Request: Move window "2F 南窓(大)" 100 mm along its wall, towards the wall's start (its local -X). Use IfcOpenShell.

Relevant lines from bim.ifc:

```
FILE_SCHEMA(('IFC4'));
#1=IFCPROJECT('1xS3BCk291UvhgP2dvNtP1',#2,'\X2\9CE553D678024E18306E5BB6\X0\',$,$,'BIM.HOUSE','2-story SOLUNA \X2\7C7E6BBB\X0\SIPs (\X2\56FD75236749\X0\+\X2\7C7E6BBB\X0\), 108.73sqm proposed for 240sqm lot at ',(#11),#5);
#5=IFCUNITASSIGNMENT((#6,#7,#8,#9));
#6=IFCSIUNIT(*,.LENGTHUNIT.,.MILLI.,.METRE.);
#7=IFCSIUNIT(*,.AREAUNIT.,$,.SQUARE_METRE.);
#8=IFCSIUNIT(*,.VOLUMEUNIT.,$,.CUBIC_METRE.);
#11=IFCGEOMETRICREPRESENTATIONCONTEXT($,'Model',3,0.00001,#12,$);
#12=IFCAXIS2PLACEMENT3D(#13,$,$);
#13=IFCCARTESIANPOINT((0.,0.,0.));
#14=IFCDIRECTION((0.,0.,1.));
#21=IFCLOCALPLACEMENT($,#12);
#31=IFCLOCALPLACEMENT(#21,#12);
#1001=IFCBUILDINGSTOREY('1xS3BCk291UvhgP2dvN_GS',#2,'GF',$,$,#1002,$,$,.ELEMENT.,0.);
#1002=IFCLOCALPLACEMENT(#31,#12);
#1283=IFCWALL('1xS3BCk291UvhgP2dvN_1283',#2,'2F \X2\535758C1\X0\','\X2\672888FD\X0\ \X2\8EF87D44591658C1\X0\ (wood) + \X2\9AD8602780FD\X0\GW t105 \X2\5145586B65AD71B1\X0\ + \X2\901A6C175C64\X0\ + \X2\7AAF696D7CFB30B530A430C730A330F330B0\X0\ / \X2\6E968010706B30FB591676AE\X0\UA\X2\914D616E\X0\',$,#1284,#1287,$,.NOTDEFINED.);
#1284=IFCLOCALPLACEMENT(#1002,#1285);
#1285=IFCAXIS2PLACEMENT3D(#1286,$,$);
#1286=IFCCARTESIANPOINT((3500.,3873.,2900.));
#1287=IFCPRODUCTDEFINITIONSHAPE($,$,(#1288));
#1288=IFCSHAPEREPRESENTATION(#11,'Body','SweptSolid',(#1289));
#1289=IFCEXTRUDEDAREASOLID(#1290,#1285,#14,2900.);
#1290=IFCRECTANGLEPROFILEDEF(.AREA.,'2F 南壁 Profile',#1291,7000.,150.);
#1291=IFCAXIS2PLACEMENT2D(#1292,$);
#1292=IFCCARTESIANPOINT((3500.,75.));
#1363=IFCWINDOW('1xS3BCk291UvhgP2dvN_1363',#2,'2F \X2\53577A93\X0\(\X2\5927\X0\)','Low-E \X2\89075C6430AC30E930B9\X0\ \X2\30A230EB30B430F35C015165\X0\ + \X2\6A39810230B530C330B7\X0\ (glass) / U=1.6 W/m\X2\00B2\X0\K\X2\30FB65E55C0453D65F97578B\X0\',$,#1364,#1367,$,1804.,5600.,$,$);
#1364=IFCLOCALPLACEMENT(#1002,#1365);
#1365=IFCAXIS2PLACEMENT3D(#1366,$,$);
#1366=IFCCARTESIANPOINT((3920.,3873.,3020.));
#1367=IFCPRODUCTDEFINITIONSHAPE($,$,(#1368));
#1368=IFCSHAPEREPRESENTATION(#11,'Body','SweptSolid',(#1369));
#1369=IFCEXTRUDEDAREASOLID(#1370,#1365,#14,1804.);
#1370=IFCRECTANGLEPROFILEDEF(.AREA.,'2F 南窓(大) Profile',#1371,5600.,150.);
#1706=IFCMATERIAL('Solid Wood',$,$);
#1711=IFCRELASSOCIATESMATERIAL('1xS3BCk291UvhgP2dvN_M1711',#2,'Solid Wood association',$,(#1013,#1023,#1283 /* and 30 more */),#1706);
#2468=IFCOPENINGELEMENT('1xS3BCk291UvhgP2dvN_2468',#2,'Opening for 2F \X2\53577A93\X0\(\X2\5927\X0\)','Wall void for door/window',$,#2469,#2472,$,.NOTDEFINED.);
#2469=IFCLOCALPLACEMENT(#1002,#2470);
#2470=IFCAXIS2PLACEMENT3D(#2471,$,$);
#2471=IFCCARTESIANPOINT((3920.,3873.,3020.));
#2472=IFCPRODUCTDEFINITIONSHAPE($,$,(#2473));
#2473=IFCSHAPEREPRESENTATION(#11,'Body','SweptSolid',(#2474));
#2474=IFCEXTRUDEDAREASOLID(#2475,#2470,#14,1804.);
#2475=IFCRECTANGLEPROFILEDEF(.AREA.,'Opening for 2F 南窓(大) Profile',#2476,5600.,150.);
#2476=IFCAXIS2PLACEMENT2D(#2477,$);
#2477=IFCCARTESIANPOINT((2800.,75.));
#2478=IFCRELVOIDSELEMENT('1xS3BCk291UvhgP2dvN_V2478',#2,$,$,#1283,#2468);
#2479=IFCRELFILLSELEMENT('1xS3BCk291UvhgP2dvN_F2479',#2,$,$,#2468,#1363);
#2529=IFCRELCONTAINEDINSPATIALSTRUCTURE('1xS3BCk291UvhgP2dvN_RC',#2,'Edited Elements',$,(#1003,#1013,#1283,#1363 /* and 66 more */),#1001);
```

```python
import ifcopenshell
import ifcopenshell.api.geometry
import ifcopenshell.util.placement

model = ifcopenshell.open("bim.ifc")

window = model.by_guid("1xS3BCk291UvhgP2dvN_1363")
opening = window.FillsVoids[0].RelatingOpeningElement
wall = opening.VoidsElements[0].RelatingBuildingElement

wall_matrix = ifcopenshell.util.placement.get_local_placement(wall.ObjectPlacement)
shift = wall_matrix[:3, 0] * -100.0
before = ifcopenshell.util.placement.get_local_placement(window.ObjectPlacement)[:3, 3].copy()

# The window is not placed relative to its opening, so move both.
for product in (opening, window):
    matrix = ifcopenshell.util.placement.get_local_placement(product.ObjectPlacement)
    matrix[:3, 3] += shift
    ifcopenshell.api.geometry.edit_object_placement(model, product=product, matrix=matrix, is_si=False)

after = ifcopenshell.util.placement.get_local_placement(window.ObjectPlacement)[:3, 3]
print("window moved by", (after - before).round(3) + 0.0)

model.write("bim_updated.ifc")
```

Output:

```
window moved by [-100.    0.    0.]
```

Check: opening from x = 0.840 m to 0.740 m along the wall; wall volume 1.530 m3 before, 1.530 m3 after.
